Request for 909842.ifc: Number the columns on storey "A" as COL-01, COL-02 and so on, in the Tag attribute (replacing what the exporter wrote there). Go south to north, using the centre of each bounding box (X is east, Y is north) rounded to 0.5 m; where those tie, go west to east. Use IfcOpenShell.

First a look at what the model holds.

```python
import ifcopenshell
import ifcopenshell.util.element
import ifcopenshell.util.placement

model = ifcopenshell.open("909842.ifc")
print(model.schema)
storey = next(s for s in model.by_type("IfcBuildingStorey") if s.Name == "A")
columns = [e for e in ifcopenshell.util.element.get_decomposition(storey) if e.is_a("IfcColumn")]
for e in sorted(columns, key=lambda e: e.id()):
    origin = ifcopenshell.util.placement.get_local_placement(e.ObjectPlacement)[:3, 3]
    print(e.id(), e.Tag, e.Name, origin.round(2) + 0.0, sep=" | ")
```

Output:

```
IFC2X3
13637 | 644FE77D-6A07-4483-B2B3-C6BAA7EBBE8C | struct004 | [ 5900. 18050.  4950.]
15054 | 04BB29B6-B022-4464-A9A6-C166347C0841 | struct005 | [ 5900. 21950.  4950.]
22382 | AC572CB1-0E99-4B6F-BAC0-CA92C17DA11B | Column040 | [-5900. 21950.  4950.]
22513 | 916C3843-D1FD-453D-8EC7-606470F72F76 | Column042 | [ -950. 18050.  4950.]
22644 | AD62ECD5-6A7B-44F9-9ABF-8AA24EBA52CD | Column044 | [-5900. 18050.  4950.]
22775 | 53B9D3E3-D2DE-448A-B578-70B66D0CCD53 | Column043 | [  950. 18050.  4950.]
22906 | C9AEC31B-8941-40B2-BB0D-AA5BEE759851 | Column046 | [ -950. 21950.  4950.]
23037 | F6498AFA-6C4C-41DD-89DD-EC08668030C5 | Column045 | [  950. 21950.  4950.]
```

```python
import ifcopenshell
import ifcopenshell.geom
import ifcopenshell.util.element
import ifcopenshell.util.shape

model = ifcopenshell.open("909842.ifc")
settings = ifcopenshell.geom.settings()
settings.set("use-world-coords", True)


def centre(element):
    shape = ifcopenshell.geom.create_shape(settings, element)
    return ifcopenshell.util.shape.get_bbox_centroid(shape.geometry)


storey = next(s for s in model.by_type("IfcBuildingStorey") if s.Name == "A")
columns = [e for e in ifcopenshell.util.element.get_decomposition(storey) if e.is_a("IfcColumn")]

# Insertion points can sit at a corner or the storey origin, so sort by the geometry (in metres).
centres = {e: centre(e) for e in columns}
columns.sort(key=lambda e: (round(centres[e][1] / 0.5), centres[e][0]))

for i, e in enumerate(columns, start=1):
    number = f"COL-{i:02d}"
    e.Tag = number
    print(e.id(), number)

model.write("909842_edited.ifc")
```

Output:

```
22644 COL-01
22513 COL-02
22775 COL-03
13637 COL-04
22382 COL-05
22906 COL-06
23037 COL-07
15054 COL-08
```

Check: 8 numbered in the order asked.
